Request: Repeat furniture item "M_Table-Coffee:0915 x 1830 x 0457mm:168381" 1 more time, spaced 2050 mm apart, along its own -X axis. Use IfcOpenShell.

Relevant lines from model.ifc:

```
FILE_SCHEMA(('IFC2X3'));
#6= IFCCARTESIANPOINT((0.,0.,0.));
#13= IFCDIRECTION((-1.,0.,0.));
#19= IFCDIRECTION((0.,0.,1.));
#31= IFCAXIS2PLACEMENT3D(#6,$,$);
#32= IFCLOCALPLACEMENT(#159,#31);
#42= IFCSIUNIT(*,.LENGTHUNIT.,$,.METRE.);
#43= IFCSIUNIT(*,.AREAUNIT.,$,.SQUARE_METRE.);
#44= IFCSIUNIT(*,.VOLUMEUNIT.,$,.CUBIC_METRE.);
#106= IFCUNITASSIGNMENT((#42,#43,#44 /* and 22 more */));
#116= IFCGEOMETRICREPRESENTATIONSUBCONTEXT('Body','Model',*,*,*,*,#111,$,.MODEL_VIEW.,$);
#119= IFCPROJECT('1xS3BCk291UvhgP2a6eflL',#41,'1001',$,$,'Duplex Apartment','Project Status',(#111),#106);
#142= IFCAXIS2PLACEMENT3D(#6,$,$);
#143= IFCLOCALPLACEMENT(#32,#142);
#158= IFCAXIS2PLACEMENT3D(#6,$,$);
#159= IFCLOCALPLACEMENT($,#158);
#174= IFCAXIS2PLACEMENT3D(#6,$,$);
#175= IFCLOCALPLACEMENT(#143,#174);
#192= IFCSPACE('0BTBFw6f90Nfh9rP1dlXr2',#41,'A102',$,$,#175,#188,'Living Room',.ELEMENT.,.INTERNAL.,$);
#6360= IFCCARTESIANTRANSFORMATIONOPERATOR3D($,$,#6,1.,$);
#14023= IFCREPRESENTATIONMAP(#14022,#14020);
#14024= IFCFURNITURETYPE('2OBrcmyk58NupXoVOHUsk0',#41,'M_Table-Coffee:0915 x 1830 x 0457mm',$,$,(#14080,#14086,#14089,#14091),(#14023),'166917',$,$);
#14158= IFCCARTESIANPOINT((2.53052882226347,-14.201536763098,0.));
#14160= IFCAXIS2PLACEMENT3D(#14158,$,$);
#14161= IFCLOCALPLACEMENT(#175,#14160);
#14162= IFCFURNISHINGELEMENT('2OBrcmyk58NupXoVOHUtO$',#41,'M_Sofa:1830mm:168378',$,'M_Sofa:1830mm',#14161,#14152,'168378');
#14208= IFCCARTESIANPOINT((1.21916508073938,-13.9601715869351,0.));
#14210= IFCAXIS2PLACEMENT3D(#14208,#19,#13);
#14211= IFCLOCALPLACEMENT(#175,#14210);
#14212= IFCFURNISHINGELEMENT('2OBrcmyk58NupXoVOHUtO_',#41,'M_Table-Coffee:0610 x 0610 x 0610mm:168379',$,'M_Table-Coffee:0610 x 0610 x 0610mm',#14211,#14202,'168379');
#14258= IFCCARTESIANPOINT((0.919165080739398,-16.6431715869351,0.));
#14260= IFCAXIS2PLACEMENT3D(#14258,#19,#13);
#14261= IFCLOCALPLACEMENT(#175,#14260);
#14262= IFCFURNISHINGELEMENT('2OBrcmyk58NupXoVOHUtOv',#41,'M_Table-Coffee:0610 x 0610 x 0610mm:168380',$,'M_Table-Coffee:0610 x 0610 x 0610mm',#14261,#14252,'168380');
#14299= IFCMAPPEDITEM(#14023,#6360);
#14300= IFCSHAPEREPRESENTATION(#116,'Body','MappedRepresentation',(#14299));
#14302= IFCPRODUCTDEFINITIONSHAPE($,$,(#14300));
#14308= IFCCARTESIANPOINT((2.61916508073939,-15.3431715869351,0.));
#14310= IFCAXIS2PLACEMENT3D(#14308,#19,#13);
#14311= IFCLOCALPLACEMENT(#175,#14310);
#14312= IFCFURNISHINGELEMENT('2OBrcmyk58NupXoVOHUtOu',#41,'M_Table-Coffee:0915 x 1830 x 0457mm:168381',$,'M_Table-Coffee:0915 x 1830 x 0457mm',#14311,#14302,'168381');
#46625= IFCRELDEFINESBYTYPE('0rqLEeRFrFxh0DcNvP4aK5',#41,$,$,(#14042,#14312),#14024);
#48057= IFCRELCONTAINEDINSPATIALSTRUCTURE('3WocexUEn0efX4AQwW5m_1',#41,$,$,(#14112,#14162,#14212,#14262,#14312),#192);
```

```python
import ifcopenshell
import ifcopenshell.api.geometry
import ifcopenshell.api.root
import ifcopenshell.util.element
import ifcopenshell.util.placement

model = ifcopenshell.open("model.ifc")


def reuse_history(source, copy):
    """copy_class also copies each property set's owner history, people and application; keep the originals."""
    for rel in copy.IsDefinedBy:
        if rel.is_a("IfcRelDefinesByProperties") and (history := rel.RelatingPropertyDefinition.OwnerHistory):
            rel.RelatingPropertyDefinition.OwnerHistory = source.OwnerHistory
            ifcopenshell.util.element.remove_deep2(model, history)


source = model.by_guid("2OBrcmyk58NupXoVOHUtOu")
base = ifcopenshell.util.placement.get_local_placement(source.ObjectPlacement)
step = -base[:3, 0] * 2.05

for i in range(1, 2):
    copy = ifcopenshell.api.root.copy_class(model, product=source)
    copy.Representation = ifcopenshell.util.element.copy_deep(
        model, source.Representation, exclude=["IfcGeometricRepresentationContext", "IfcRepresentationMap"]
    )
    copy.Name = "M_Table-Coffee:0915 x 1830 x 0457mm"
    copy.Tag = None
    reuse_history(source, copy)
    matrix = base.copy()
    matrix[:3, 3] += i * step
    print("added at", matrix[:3, 3].round(3) + 0.0)
    ifcopenshell.api.geometry.edit_object_placement(model, product=copy, matrix=matrix, is_si=False)

model.write("model_rev.ifc")
```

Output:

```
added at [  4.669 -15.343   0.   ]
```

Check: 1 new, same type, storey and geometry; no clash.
